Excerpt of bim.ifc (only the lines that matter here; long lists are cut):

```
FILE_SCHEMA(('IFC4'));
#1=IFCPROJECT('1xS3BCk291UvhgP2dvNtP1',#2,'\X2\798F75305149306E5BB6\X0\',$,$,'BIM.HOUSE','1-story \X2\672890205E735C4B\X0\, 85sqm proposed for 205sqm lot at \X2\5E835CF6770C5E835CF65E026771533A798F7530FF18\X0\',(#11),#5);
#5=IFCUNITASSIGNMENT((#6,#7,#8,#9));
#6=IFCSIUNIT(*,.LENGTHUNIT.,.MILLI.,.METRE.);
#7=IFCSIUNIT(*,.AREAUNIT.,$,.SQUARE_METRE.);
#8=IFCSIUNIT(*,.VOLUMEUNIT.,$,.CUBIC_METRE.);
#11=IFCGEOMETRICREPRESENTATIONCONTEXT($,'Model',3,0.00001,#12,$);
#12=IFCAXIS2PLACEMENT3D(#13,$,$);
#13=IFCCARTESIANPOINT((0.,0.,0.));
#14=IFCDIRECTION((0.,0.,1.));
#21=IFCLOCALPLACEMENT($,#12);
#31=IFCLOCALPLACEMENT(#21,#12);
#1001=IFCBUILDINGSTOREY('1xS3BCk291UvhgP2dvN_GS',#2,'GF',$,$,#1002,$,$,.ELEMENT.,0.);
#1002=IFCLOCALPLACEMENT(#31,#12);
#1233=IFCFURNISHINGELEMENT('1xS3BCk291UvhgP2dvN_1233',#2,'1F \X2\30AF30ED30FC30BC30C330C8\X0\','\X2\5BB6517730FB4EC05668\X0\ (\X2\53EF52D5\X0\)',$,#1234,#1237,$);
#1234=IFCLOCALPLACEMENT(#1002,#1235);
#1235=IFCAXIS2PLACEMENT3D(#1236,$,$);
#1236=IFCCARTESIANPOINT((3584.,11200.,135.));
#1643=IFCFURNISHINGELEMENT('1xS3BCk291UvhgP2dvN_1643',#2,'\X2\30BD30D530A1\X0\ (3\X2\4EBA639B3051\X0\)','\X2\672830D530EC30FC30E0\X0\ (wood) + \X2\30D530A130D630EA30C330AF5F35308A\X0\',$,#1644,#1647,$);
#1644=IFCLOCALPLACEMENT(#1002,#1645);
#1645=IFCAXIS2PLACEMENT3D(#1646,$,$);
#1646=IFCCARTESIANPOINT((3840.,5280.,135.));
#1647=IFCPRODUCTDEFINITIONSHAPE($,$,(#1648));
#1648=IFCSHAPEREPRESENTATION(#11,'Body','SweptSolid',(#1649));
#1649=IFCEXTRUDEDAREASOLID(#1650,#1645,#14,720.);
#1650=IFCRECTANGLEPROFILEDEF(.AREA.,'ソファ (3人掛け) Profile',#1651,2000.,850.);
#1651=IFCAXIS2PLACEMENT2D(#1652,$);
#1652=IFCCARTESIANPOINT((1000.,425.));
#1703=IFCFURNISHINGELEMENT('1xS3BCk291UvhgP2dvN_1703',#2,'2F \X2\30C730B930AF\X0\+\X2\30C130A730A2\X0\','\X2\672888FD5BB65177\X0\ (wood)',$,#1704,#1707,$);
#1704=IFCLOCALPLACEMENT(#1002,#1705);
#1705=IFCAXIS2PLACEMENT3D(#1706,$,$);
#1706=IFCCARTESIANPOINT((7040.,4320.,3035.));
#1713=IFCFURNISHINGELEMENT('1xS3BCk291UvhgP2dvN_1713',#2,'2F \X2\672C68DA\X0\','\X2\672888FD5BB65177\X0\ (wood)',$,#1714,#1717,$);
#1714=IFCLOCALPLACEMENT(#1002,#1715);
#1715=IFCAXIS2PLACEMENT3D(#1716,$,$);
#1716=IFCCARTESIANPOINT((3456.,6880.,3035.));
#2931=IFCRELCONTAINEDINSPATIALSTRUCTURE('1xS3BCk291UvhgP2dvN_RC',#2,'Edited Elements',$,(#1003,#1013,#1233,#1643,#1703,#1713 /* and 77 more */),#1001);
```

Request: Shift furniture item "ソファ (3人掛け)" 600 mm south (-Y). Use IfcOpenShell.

```python
import ifcopenshell
import ifcopenshell.api.geometry
import ifcopenshell.util.placement
import ifcopenshell.util.unit

model = ifcopenshell.open("bim.ifc")
unit_scale = ifcopenshell.util.unit.calculate_unit_scale(model)

item = model.by_guid("1xS3BCk291UvhgP2dvN_1643")
matrix = ifcopenshell.util.placement.get_local_placement(item.ObjectPlacement)
matrix[1, 3] -= 0.6 / unit_scale
ifcopenshell.api.geometry.edit_object_placement(model, product=item, matrix=matrix, is_si=False)

print(ifcopenshell.util.placement.get_local_placement(item.ObjectPlacement).round(3) + 0.0)

model.write("bim_updated.ifc")
```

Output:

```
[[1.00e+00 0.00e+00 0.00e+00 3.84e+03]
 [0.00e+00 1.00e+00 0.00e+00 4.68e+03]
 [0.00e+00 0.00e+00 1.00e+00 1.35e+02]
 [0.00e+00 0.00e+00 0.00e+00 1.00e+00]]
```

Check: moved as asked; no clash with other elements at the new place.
